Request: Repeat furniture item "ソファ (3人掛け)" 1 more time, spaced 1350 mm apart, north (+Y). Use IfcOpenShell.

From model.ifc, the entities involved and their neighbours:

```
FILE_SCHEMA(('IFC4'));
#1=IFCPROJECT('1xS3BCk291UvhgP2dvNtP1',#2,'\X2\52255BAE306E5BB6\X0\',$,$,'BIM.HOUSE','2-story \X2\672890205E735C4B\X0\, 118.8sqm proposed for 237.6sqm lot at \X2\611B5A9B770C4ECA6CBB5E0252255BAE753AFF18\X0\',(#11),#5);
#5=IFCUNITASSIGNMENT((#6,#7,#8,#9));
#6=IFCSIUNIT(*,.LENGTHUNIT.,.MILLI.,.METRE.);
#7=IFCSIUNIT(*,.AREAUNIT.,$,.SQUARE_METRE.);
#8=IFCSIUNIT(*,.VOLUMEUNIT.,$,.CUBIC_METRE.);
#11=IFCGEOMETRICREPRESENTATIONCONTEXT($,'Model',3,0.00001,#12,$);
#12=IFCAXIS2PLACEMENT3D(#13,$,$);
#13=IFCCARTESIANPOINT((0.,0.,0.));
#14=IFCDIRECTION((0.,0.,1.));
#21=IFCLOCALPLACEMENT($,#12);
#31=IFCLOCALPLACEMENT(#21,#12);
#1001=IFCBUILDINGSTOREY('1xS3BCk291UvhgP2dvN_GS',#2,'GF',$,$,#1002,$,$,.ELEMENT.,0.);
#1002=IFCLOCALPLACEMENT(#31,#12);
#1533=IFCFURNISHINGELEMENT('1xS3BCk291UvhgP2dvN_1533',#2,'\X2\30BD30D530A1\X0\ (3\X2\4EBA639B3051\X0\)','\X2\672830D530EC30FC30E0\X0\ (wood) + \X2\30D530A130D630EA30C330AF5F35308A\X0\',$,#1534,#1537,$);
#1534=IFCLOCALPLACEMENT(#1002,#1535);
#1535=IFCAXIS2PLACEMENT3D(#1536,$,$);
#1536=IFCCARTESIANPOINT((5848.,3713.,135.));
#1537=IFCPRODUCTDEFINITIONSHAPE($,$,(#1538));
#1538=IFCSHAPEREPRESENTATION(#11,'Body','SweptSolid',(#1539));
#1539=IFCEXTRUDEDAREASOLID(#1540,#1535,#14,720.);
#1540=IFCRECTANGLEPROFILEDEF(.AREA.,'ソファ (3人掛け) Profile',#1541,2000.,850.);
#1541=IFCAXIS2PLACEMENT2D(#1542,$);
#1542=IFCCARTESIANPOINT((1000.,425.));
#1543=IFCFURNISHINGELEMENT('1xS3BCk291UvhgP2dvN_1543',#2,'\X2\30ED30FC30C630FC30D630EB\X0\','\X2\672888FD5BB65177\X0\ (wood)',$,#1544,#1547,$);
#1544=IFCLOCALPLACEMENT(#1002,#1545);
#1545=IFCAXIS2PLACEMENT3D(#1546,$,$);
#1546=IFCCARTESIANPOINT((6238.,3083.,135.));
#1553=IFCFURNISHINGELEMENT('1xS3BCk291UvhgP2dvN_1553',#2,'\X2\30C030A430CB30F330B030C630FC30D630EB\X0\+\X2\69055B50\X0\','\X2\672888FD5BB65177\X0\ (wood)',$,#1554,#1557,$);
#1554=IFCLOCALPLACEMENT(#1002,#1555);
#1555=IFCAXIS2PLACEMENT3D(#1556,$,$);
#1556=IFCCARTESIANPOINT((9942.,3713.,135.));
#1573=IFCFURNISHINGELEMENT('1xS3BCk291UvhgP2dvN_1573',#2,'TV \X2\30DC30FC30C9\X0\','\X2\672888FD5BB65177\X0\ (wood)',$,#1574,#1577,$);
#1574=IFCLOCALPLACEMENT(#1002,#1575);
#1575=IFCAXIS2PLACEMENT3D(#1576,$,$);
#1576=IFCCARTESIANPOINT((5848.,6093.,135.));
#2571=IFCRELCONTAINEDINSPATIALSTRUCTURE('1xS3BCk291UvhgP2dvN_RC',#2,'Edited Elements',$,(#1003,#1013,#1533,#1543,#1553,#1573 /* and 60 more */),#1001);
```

```python
import numpy as np
import ifcopenshell
import ifcopenshell.api.geometry
import ifcopenshell.api.root
import ifcopenshell.util.element
import ifcopenshell.util.placement
import ifcopenshell.util.unit

model = ifcopenshell.open("model.ifc")
unit_scale = ifcopenshell.util.unit.calculate_unit_scale(model)


def reuse_history(source, copy):
    """copy_class also copies each property set's owner history, people and application; keep the originals."""
    for rel in copy.IsDefinedBy:
        if rel.is_a("IfcRelDefinesByProperties") and (history := rel.RelatingPropertyDefinition.OwnerHistory):
            rel.RelatingPropertyDefinition.OwnerHistory = source.OwnerHistory
            ifcopenshell.util.element.remove_deep2(model, history)


source = model.by_id(1533)
base = ifcopenshell.util.placement.get_local_placement(source.ObjectPlacement)
step = np.array([0.0, 1.0, 0.0]) * 1.35 / unit_scale

for i in range(1, 2):
    copy = ifcopenshell.api.root.copy_class(model, product=source)
    copy.Representation = ifcopenshell.util.element.copy_deep(
        model, source.Representation, exclude=["IfcGeometricRepresentationContext", "IfcRepresentationMap"]
    )
    reuse_history(source, copy)
    matrix = base.copy()
    matrix[:3, 3] += i * step
    print("added at", matrix[:3, 3].round(3) + 0.0)
    ifcopenshell.api.geometry.edit_object_placement(model, product=copy, matrix=matrix, is_si=False)

model.write("model_v2.ifc")
```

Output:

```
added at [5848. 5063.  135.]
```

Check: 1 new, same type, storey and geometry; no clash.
